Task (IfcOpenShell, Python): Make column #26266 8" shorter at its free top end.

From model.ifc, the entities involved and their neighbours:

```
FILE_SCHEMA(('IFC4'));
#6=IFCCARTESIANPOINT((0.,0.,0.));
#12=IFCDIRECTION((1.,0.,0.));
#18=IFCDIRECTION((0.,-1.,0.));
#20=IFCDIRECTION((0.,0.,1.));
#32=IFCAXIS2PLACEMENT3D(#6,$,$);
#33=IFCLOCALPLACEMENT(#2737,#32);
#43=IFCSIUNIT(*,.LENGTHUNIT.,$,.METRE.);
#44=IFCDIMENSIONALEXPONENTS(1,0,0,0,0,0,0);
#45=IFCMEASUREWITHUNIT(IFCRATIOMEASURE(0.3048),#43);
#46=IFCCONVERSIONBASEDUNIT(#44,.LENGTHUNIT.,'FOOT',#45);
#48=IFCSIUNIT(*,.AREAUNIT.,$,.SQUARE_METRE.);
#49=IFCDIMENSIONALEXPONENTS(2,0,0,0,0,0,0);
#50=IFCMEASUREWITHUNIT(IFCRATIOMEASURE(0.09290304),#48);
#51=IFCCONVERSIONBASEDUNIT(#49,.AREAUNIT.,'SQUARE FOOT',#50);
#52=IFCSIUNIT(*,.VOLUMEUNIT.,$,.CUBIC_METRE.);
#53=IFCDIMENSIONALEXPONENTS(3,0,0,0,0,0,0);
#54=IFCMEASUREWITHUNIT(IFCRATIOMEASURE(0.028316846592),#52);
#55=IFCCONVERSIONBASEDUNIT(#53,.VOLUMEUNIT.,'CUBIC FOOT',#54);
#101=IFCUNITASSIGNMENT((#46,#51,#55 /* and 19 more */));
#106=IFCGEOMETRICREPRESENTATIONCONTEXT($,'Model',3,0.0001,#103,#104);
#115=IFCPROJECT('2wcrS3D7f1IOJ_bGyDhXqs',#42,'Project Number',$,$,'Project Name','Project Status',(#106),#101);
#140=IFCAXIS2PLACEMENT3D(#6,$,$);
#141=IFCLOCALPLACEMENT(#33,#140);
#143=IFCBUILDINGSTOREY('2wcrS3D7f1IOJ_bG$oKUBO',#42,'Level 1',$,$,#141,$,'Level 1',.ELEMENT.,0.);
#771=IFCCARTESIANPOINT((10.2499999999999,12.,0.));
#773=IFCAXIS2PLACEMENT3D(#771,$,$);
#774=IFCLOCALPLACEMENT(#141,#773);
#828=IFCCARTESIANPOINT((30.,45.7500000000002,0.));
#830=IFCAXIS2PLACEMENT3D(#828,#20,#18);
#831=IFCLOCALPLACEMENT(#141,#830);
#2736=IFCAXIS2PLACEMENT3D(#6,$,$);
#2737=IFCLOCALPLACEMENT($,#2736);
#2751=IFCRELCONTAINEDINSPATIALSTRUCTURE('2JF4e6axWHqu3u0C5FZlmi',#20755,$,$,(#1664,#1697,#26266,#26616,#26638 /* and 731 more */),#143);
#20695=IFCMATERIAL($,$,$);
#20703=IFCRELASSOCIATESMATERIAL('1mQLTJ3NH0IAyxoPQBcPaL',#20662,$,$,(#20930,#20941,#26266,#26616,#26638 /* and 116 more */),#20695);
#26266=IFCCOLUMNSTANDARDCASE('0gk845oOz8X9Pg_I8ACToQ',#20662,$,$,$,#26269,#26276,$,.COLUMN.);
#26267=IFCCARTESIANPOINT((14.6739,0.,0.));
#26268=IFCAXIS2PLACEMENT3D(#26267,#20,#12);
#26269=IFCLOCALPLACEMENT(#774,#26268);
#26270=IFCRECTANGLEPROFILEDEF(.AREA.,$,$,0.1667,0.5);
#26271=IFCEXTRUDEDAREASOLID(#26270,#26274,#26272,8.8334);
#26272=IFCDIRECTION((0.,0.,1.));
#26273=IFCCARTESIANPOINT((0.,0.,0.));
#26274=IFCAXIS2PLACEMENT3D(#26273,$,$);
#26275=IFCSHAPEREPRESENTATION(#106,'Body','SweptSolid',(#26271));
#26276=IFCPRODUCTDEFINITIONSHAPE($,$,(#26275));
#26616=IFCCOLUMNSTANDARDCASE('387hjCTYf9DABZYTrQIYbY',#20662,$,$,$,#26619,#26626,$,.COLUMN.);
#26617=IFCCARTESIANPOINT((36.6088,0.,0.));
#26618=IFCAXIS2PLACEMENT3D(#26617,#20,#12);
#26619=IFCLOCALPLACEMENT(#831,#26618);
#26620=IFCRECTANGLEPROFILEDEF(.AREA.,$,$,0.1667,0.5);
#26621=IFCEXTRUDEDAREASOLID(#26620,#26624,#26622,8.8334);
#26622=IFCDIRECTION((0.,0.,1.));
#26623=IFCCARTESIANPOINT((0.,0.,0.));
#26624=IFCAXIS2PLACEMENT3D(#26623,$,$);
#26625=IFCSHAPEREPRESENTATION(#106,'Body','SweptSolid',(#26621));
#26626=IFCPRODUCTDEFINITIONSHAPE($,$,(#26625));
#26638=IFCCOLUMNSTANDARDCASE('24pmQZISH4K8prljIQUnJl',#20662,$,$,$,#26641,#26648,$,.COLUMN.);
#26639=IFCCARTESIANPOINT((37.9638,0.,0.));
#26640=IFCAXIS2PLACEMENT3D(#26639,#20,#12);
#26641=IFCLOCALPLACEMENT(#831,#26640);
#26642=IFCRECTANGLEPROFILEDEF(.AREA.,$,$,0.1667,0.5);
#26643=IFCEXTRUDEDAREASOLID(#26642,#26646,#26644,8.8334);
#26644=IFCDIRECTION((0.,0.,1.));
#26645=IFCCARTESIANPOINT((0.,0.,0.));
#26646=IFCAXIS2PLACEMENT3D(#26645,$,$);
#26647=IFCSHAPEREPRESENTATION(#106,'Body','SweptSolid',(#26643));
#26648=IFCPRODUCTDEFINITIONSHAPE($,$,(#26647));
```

```python
import ifcopenshell
import ifcopenshell.util.unit

model = ifcopenshell.open("model.ifc")
unit_scale = ifcopenshell.util.unit.calculate_unit_scale(model)

member = model.by_guid("0gk845oOz8X9Pg_I8ACToQ")
change = -8 * 0.0254 / unit_scale

# The extrusion runs towards the end named, so only its depth changes.
body = next(r for r in member.Representation.Representations if r.RepresentationIdentifier == "Body")
solid = body.Items[0]
old_length = solid.Depth
solid.Depth += change

print(f"length {old_length:g} -> {solid.Depth:g}")

model.write("model_rev.ifc")
```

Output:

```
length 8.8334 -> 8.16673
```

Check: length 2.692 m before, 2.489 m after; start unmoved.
